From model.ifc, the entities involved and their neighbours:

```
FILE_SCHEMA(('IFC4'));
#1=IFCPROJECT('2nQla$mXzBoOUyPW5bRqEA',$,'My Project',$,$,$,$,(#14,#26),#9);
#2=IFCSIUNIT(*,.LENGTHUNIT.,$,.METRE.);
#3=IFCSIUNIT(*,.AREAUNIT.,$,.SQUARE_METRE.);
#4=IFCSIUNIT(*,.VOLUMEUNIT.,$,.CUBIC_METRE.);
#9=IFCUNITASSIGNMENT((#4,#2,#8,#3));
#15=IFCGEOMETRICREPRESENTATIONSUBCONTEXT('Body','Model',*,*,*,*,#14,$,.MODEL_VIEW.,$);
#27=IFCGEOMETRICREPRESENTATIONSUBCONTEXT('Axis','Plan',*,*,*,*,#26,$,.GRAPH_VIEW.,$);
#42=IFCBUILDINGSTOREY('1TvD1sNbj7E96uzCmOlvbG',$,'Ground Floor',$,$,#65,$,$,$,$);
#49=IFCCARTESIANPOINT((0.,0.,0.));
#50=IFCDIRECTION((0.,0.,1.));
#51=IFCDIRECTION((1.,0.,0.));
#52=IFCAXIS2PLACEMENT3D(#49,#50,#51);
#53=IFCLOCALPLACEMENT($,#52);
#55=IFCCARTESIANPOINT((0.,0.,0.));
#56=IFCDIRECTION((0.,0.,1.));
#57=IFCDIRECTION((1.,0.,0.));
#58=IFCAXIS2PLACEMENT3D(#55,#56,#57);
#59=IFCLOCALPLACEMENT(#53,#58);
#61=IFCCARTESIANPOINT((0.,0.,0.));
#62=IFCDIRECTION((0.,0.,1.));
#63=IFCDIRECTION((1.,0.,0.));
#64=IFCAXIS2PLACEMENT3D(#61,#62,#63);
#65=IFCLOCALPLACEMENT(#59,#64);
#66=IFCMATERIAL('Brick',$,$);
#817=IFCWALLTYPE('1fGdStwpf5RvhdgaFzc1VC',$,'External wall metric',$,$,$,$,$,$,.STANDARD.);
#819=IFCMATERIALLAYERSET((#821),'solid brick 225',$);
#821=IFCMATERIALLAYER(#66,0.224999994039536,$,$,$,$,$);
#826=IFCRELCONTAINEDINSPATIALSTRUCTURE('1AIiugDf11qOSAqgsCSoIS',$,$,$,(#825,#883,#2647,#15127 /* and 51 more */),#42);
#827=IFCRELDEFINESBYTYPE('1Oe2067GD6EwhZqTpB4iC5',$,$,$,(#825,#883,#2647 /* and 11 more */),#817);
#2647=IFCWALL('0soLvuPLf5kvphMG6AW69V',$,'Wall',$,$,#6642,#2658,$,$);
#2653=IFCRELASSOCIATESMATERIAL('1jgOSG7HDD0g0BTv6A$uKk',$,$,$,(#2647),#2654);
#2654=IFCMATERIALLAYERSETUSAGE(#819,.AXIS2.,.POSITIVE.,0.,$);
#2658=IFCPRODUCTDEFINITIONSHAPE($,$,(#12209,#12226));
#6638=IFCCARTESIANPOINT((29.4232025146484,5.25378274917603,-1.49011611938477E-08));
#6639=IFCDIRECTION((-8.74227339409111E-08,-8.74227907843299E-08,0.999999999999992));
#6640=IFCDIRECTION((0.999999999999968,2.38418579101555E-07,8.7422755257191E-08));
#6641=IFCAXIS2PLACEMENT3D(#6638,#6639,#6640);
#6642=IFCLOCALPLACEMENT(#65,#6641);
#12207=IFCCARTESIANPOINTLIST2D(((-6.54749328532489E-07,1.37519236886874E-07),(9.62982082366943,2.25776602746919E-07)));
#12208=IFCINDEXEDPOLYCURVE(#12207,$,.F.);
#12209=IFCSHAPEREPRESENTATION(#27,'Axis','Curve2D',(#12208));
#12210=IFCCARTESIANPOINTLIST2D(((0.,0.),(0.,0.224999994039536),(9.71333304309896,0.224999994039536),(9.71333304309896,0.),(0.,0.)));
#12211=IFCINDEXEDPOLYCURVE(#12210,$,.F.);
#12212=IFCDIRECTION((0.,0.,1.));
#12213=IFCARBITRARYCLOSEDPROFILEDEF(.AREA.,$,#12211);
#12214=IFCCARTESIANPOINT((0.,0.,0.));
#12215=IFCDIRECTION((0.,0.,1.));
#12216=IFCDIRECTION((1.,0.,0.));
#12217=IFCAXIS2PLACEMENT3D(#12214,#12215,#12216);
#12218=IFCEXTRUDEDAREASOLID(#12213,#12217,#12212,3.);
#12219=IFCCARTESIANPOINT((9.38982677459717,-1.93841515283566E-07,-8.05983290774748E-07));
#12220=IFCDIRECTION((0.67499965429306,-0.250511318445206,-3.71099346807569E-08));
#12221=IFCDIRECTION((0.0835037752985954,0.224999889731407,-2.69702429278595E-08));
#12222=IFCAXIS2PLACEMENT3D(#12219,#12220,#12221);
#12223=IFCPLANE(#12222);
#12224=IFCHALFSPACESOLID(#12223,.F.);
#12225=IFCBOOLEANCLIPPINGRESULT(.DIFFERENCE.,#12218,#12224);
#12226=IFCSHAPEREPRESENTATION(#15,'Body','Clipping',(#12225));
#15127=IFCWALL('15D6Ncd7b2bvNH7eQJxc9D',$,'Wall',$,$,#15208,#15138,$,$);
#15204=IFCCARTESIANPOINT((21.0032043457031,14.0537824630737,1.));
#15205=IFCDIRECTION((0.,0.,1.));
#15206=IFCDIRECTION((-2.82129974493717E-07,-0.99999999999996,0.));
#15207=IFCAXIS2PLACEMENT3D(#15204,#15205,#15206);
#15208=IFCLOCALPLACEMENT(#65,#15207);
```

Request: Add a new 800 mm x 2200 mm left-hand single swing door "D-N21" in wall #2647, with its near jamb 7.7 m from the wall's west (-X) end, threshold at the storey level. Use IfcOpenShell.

```python
import numpy as np
import ifcopenshell
import ifcopenshell.api.feature
import ifcopenshell.api.geometry
import ifcopenshell.api.root
import ifcopenshell.api.spatial
import ifcopenshell.geom
import ifcopenshell.util.element
import ifcopenshell.util.placement
import ifcopenshell.util.representation
import ifcopenshell.util.shape
import ifcopenshell.util.unit

model = ifcopenshell.open("model.ifc")
unit_scale = ifcopenshell.util.unit.calculate_unit_scale(model)
settings = ifcopenshell.geom.settings()


def volume(element):
    """Net volume in cubic metres, openings subtracted."""
    shape = ifcopenshell.geom.create_shape(settings, element)
    return ifcopenshell.util.shape.get_volume(shape.geometry)


wall = model.by_guid("0soLvuPLf5kvphMG6AW69V")
storey = ifcopenshell.util.element.get_container(wall, ifc_class="IfcBuildingStorey")
context = ifcopenshell.util.representation.get_context(model, "Model", "Body", "MODEL_VIEW")
before = volume(wall)

width, height, from_end, sill = 0.8, 2.2, 7.7, 0.0  # metres

# The wall runs along its own X axis, and the end named is its -X end.
wall_shape = ifcopenshell.geom.create_shape(settings, wall)
x, y, z = ifcopenshell.util.shape.get_vertices(wall_shape.geometry).T
start = x.min() + from_end
face, thickness = float(y.min()), float(y.max() - y.min())
wall_matrix = ifcopenshell.util.placement.get_local_placement(wall.ObjectPlacement)
level = ifcopenshell.util.placement.get_local_placement(storey.ObjectPlacement)[2, 3]


def in_wall(x, y):
    """Placement at x, y metres in the wall's axes, at sill height."""
    matrix = wall_matrix.copy()
    matrix[:, 3] = wall_matrix @ np.array([x / unit_scale, y / unit_scale, 0.0, 1.0])
    matrix[2, 3] = level + sill / unit_scale
    return matrix


# Opening: a box that overshoots both wall faces by 50 mm.
opening = ifcopenshell.api.root.create_entity(model, ifc_class="IfcOpeningElement", predefined_type="OPENING")
box = ifcopenshell.api.geometry.add_wall_representation(
    model, context=context, length=width, height=height, thickness=thickness + 0.1
)
ifcopenshell.api.geometry.assign_representation(model, product=opening, representation=box)
ifcopenshell.api.geometry.edit_object_placement(model, product=opening, matrix=in_wall(start, face - 0.05), is_si=False)
ifcopenshell.api.feature.add_feature(model, feature=opening, element=wall)

door = ifcopenshell.api.root.create_entity(model, ifc_class="IfcDoor", name="D-N21", predefined_type="DOOR")
door.OverallWidth, door.OverallHeight = width / unit_scale, height / unit_scale
door.OperationType = "SINGLE_SWING_LEFT"
body = ifcopenshell.api.geometry.add_door_representation(
    model,
    context=context,
    overall_width=door.OverallWidth,
    overall_height=door.OverallHeight,
    operation_type="SINGLE_SWING_LEFT",
    lining_properties={"LiningDepth": thickness / unit_scale, "ThresholdDepth": thickness / unit_scale},
)
ifcopenshell.api.geometry.assign_representation(model, product=door, representation=body)
ifcopenshell.api.spatial.assign_container(model, products=[door], relating_structure=storey)
ifcopenshell.api.feature.add_filling(model, opening=opening, element=door)

# The lining spans the wall, so the door starts at the wall face.
ifcopenshell.api.geometry.edit_object_placement(model, product=door, matrix=in_wall(start, face), is_si=False)

after = volume(wall)

print(f"wall volume {before:.3f} -> {after:.3f} m3")

model.write("model-out.ifc")
```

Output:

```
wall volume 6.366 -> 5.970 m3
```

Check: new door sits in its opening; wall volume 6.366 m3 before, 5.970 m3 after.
